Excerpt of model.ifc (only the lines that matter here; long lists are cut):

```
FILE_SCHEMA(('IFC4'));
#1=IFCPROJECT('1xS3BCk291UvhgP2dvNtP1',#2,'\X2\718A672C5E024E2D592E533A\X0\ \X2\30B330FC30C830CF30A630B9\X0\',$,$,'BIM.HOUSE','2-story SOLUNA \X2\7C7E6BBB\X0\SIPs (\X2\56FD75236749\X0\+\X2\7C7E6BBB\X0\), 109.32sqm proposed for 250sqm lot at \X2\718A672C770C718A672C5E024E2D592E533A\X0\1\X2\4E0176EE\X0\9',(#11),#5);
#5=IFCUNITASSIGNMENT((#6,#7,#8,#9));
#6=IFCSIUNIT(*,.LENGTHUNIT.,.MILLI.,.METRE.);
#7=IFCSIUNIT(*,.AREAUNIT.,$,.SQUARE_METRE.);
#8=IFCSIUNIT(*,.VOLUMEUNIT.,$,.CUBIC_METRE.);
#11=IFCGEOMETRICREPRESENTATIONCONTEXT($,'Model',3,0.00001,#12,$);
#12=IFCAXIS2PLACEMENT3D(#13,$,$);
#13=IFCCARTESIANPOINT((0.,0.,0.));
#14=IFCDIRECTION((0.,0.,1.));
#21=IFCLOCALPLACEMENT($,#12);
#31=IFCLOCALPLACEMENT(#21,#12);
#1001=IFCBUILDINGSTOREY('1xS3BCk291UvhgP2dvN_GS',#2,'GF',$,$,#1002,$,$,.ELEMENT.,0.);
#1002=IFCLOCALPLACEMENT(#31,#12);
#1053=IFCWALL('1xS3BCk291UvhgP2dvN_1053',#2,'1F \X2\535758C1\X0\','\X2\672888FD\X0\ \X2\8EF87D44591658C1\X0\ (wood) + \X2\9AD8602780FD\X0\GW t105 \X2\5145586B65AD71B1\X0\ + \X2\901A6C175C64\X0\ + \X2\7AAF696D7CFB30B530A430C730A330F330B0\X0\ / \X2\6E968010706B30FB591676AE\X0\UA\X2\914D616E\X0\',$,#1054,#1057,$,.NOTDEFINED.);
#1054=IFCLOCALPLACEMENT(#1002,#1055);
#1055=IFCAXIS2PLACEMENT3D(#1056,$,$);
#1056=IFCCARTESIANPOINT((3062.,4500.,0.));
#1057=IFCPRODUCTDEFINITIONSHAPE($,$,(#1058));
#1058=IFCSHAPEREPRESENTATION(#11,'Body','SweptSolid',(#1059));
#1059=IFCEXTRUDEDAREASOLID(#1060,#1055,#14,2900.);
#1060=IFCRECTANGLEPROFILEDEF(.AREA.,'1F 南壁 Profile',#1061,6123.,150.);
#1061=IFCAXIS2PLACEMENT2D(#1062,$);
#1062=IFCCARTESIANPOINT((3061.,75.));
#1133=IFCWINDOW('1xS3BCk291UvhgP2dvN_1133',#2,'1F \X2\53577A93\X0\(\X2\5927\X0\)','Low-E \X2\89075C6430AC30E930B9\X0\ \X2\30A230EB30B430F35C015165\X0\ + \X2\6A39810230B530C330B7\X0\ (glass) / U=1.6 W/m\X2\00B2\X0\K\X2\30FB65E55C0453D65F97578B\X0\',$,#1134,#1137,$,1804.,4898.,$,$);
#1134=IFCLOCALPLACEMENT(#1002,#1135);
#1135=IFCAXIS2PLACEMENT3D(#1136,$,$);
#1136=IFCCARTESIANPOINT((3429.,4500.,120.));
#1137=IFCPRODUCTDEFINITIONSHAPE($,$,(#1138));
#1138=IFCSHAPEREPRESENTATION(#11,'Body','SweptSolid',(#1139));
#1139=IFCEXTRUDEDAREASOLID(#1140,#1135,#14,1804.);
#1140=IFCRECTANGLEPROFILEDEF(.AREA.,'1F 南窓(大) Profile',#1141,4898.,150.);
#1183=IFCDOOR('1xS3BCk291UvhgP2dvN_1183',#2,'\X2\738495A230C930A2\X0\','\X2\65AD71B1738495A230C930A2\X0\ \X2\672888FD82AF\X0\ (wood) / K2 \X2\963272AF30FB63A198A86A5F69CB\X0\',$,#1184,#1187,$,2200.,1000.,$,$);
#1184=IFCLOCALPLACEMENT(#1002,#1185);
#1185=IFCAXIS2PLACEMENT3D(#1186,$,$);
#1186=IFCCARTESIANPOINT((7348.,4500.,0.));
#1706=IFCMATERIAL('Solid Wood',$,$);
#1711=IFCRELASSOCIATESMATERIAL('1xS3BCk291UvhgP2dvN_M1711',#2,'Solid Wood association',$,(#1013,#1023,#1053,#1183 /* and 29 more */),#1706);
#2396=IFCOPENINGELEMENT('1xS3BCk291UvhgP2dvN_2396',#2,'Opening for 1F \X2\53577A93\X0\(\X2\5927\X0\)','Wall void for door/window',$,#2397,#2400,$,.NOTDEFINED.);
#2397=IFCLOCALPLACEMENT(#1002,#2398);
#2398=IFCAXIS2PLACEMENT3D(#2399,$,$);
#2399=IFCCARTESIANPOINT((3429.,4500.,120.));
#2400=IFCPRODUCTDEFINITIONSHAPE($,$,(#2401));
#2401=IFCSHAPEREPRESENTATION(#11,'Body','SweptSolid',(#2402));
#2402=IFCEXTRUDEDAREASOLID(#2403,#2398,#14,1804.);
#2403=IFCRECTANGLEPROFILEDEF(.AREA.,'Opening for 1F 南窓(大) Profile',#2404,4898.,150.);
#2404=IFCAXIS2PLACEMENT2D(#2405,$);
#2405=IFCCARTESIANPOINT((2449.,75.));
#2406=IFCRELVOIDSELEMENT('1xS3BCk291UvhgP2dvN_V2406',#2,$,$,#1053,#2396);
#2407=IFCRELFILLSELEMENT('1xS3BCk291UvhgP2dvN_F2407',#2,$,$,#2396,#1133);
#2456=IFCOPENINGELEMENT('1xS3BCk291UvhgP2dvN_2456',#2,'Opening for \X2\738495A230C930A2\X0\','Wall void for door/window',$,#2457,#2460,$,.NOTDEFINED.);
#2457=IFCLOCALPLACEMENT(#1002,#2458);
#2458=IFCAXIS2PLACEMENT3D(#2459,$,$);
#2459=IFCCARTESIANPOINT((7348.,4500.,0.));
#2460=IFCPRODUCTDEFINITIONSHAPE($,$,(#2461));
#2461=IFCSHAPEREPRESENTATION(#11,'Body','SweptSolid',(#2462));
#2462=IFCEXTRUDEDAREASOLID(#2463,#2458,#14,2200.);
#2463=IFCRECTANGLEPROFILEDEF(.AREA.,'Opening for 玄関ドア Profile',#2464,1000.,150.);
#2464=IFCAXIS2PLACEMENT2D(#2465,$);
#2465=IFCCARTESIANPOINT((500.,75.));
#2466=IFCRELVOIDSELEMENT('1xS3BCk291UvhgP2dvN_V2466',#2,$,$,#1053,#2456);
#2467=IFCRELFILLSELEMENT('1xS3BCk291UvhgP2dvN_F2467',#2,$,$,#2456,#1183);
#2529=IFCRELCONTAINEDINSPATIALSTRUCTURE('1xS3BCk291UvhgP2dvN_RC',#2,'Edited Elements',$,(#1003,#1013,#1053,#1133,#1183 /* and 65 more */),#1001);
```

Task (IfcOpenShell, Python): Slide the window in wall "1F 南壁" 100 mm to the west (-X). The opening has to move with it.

```python
import ifcopenshell
import ifcopenshell.api.geometry
import ifcopenshell.util.placement

model = ifcopenshell.open("model.ifc")

window = model.by_id(1133)
opening = window.FillsVoids[0].RelatingOpeningElement
wall = opening.VoidsElements[0].RelatingBuildingElement

wall_matrix = ifcopenshell.util.placement.get_local_placement(wall.ObjectPlacement)
shift = wall_matrix[:3, 0] * -100.0
before = ifcopenshell.util.placement.get_local_placement(window.ObjectPlacement)[:3, 3].copy()

# The window is not placed relative to its opening, so move both.
for product in (opening, window):
    matrix = ifcopenshell.util.placement.get_local_placement(product.ObjectPlacement)
    matrix[:3, 3] += shift
    ifcopenshell.api.geometry.edit_object_placement(model, product=product, matrix=matrix, is_si=False)

after = ifcopenshell.util.placement.get_local_placement(window.ObjectPlacement)[:3, 3]
print("window moved by", (after - before).round(3) + 0.0)

model.write("model_updated.ifc")
```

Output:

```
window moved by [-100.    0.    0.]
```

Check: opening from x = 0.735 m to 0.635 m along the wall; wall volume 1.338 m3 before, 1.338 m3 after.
